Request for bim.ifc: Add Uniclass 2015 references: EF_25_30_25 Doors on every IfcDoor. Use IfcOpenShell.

First a look at what the model holds.

```python
import ifcopenshell

model = ifcopenshell.open("bim.ifc")
print(model.schema)
print("classifications:", [c.Name for c in model.by_type("IfcClassification")])
for ifc_class in ("IfcDoor", "IfcRoof", "IfcStair", "IfcWall", "IfcWindow"):
    print(ifc_class, len(model.by_type(ifc_class)))
```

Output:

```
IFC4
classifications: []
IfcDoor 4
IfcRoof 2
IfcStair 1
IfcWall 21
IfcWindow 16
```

```python
import ifcopenshell
import ifcopenshell.api.classification

model = ifcopenshell.open("bim.ifc")

system = ifcopenshell.api.classification.add_classification(model, classification="Uniclass 2015")

codes = {
    "IfcDoor": ("EF_25_30_25", "Doors"),
}
for ifc_class, (code, name) in codes.items():
    products = model.by_type(ifc_class)
    ifcopenshell.api.classification.add_reference(
        model, products=products, classification=system, identification=code, name=name
    )
    print(code, len(products))

model.write("bim_updated.ifc")
```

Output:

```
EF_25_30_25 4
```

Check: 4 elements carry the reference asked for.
